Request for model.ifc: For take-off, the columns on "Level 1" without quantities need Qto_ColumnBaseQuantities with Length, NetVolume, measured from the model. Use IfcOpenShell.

First a look at what the model holds.

```python
import ifcopenshell
import ifcopenshell.util.element
import ifcopenshell.util.unit

model = ifcopenshell.open("model.ifc")
print(model.schema)
for unit_type in ("LENGTHUNIT", "AREAUNIT", "VOLUMEUNIT"):
    print(unit_type, ifcopenshell.util.unit.calculate_unit_scale(model, unit_type))
storey = next(s for s in model.by_type("IfcBuildingStorey") if s.Name == "Level 1")
columns = [e for e in ifcopenshell.util.element.get_decomposition(storey) if e.is_a("IfcColumn")]
for e in sorted(columns, key=lambda e: e.id()):
    print(e.id(), e.is_a(), e.Name, list(ifcopenshell.util.element.get_psets(e, qtos_only=True)), sep=" | ")
```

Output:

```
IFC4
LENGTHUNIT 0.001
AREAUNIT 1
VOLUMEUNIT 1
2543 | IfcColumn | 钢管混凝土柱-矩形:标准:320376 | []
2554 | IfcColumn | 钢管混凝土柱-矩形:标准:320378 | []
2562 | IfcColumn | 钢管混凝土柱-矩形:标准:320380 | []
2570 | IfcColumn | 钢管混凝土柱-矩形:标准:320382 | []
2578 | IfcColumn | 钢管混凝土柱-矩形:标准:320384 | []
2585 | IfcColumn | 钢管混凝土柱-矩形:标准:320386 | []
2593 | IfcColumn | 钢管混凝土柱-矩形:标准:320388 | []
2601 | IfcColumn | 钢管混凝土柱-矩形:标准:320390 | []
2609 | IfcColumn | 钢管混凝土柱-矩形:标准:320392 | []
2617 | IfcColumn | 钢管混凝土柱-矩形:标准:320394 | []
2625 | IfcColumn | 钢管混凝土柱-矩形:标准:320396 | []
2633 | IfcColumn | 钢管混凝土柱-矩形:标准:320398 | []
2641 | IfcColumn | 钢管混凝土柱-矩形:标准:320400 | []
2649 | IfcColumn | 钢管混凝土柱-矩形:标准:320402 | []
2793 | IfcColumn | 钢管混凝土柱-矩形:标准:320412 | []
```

```python
import ifcopenshell
import ifcopenshell.api.pset
import ifcopenshell.geom
import ifcopenshell.util.element
import ifcopenshell.util.shape
import ifcopenshell.util.unit

model = ifcopenshell.open("model.ifc")
unit_scale = ifcopenshell.util.unit.calculate_unit_scale(model)
volume_scale = ifcopenshell.util.unit.calculate_unit_scale(model, "VOLUMEUNIT")
settings = ifcopenshell.geom.settings()

storey = next(s for s in model.by_type("IfcBuildingStorey") if s.Name == "Level 1")
columns = [e for e in ifcopenshell.util.element.get_decomposition(storey) if e.is_a("IfcColumn")]

for e in sorted(columns, key=lambda e: e.id()):
    if ifcopenshell.util.element.get_psets(e, qtos_only=True, should_inherit=False):
        continue
    # Geometry comes back in metres, in the element's own axes.
    shape = ifcopenshell.geom.create_shape(settings, e)
    values = {
        "Length": ifcopenshell.util.shape.get_z(shape.geometry) / unit_scale,
        "NetVolume": ifcopenshell.util.shape.get_volume(shape.geometry) / volume_scale,
    }
    qto = ifcopenshell.api.pset.add_qto(model, product=e, name="Qto_ColumnBaseQuantities")
    ifcopenshell.api.pset.edit_qto(model, qto=qto, properties=values)
    print(e.id(), {k: round(v, 3) for k, v in values.items()})

model.write("model_edited.ifc")
```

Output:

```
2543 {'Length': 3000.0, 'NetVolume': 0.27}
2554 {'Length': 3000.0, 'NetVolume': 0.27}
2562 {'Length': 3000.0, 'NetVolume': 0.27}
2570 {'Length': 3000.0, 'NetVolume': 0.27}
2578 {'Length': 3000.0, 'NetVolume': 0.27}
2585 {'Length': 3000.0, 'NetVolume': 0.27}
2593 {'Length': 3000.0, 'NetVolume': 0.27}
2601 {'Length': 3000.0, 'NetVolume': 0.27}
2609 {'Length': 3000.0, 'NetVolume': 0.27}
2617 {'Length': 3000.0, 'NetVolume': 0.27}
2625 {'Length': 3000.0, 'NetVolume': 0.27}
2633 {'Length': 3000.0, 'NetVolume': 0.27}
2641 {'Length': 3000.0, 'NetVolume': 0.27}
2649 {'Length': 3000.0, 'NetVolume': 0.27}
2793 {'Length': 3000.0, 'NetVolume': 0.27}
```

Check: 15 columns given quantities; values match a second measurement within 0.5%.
